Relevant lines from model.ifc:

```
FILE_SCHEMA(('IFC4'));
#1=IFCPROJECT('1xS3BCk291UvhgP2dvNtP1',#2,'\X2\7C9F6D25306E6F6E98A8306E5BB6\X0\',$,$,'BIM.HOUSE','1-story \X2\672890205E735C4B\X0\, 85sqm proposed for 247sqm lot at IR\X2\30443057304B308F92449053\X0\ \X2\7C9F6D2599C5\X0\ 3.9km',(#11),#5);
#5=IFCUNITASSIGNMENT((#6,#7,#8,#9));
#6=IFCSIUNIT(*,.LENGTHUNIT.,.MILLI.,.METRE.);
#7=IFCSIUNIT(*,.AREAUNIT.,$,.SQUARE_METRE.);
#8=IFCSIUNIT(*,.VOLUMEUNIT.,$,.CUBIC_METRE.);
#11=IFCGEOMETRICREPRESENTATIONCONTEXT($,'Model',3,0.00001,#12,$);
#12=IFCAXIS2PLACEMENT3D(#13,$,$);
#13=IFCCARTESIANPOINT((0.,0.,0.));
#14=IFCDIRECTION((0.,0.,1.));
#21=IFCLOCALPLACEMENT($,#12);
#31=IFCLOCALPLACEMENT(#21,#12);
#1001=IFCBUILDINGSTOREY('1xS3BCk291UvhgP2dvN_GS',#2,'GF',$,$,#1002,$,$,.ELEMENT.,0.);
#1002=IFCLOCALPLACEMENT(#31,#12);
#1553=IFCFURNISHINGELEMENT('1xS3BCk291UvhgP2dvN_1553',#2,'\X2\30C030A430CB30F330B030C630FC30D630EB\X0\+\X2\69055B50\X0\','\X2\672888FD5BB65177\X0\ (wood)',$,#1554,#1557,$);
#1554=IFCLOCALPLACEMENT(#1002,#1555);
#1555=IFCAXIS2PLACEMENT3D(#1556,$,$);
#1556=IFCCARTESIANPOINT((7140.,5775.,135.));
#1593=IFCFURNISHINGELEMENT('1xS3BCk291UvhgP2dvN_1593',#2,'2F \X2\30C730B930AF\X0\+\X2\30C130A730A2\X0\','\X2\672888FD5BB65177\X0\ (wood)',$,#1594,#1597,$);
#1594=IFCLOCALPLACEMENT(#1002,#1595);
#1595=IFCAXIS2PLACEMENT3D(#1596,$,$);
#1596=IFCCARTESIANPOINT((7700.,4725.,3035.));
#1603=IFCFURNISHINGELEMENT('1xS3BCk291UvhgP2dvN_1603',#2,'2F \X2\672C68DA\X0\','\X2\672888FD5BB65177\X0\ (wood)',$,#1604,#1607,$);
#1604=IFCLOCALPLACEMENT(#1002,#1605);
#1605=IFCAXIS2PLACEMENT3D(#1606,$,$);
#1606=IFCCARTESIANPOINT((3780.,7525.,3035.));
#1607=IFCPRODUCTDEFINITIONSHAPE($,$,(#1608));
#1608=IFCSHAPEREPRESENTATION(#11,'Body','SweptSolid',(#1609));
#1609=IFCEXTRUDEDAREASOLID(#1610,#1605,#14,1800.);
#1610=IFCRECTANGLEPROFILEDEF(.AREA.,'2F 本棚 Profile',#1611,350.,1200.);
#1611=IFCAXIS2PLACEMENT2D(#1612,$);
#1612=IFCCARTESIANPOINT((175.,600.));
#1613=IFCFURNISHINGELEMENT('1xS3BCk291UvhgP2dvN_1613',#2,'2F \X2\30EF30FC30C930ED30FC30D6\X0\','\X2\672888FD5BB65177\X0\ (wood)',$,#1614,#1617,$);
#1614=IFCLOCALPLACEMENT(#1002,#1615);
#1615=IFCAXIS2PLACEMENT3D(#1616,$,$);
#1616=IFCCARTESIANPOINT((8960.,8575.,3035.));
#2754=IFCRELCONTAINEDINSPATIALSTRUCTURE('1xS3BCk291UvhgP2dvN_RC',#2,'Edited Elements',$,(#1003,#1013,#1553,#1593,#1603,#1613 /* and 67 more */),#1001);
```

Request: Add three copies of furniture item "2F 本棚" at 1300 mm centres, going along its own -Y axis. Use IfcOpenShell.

```python
import ifcopenshell
import ifcopenshell.api.geometry
import ifcopenshell.api.root
import ifcopenshell.util.element
import ifcopenshell.util.placement

model = ifcopenshell.open("model.ifc")


def reuse_history(source, copy):
    """copy_class also copies each property set's owner history, people and application; keep the originals."""
    for rel in copy.IsDefinedBy:
        if rel.is_a("IfcRelDefinesByProperties") and (history := rel.RelatingPropertyDefinition.OwnerHistory):
            rel.RelatingPropertyDefinition.OwnerHistory = source.OwnerHistory
            ifcopenshell.util.element.remove_deep2(model, history)


source = model.by_guid("1xS3BCk291UvhgP2dvN_1603")
base = ifcopenshell.util.placement.get_local_placement(source.ObjectPlacement)
step = -base[:3, 1] * 1300.0

for i in range(1, 4):
    copy = ifcopenshell.api.root.copy_class(model, product=source)
    copy.Representation = ifcopenshell.util.element.copy_deep(
        model, source.Representation, exclude=["IfcGeometricRepresentationContext", "IfcRepresentationMap"]
    )
    reuse_history(source, copy)
    matrix = base.copy()
    matrix[:3, 3] += i * step
    print("added at", matrix[:3, 3].round(3) + 0.0)
    ifcopenshell.api.geometry.edit_object_placement(model, product=copy, matrix=matrix, is_si=False)

model.write("model_updated.ifc")
```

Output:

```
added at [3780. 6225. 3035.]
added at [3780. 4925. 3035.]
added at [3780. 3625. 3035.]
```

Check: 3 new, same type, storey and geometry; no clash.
